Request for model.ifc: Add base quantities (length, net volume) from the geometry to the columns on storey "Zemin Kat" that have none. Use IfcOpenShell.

First a look at what the model holds.

```python
import ifcopenshell
import ifcopenshell.util.element
import ifcopenshell.util.unit

model = ifcopenshell.open("model.ifc")
print(model.schema)
for unit_type in ("LENGTHUNIT", "AREAUNIT", "VOLUMEUNIT"):
    print(unit_type, ifcopenshell.util.unit.calculate_unit_scale(model, unit_type))
storey = next(s for s in model.by_type("IfcBuildingStorey") if s.Name == "Zemin Kat")
columns = [e for e in ifcopenshell.util.element.get_decomposition(storey) if e.is_a("IfcColumn")]
for e in sorted(columns, key=lambda e: e.id()):
    print(e.id(), e.is_a(), e.Name, list(ifcopenshell.util.element.get_psets(e, qtos_only=True)), sep=" | ")
```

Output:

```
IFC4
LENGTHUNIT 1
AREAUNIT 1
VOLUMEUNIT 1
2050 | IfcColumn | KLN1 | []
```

```python
import ifcopenshell
import ifcopenshell.api.pset
import ifcopenshell.geom
import ifcopenshell.util.element
import ifcopenshell.util.shape
import ifcopenshell.util.unit

model = ifcopenshell.open("model.ifc")
unit_scale = ifcopenshell.util.unit.calculate_unit_scale(model)
volume_scale = ifcopenshell.util.unit.calculate_unit_scale(model, "VOLUMEUNIT")
settings = ifcopenshell.geom.settings()

storey = next(s for s in model.by_type("IfcBuildingStorey") if s.Name == "Zemin Kat")
columns = [e for e in ifcopenshell.util.element.get_decomposition(storey) if e.is_a("IfcColumn")]

for e in sorted(columns, key=lambda e: e.id()):
    if ifcopenshell.util.element.get_psets(e, qtos_only=True, should_inherit=False):
        continue
    # Geometry comes back in metres, in the element's own axes.
    shape = ifcopenshell.geom.create_shape(settings, e)
    values = {
        "Length": ifcopenshell.util.shape.get_z(shape.geometry) / unit_scale,
        "NetVolume": ifcopenshell.util.shape.get_volume(shape.geometry) / volume_scale,
    }
    qto = ifcopenshell.api.pset.add_qto(model, product=e, name="Qto_ColumnBaseQuantities")
    ifcopenshell.api.pset.edit_qto(model, qto=qto, properties=values)
    print(e.id(), {k: round(v, 3) for k, v in values.items()})

model.write("model_v2.ifc")
```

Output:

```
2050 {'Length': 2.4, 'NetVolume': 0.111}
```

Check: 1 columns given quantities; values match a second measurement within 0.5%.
